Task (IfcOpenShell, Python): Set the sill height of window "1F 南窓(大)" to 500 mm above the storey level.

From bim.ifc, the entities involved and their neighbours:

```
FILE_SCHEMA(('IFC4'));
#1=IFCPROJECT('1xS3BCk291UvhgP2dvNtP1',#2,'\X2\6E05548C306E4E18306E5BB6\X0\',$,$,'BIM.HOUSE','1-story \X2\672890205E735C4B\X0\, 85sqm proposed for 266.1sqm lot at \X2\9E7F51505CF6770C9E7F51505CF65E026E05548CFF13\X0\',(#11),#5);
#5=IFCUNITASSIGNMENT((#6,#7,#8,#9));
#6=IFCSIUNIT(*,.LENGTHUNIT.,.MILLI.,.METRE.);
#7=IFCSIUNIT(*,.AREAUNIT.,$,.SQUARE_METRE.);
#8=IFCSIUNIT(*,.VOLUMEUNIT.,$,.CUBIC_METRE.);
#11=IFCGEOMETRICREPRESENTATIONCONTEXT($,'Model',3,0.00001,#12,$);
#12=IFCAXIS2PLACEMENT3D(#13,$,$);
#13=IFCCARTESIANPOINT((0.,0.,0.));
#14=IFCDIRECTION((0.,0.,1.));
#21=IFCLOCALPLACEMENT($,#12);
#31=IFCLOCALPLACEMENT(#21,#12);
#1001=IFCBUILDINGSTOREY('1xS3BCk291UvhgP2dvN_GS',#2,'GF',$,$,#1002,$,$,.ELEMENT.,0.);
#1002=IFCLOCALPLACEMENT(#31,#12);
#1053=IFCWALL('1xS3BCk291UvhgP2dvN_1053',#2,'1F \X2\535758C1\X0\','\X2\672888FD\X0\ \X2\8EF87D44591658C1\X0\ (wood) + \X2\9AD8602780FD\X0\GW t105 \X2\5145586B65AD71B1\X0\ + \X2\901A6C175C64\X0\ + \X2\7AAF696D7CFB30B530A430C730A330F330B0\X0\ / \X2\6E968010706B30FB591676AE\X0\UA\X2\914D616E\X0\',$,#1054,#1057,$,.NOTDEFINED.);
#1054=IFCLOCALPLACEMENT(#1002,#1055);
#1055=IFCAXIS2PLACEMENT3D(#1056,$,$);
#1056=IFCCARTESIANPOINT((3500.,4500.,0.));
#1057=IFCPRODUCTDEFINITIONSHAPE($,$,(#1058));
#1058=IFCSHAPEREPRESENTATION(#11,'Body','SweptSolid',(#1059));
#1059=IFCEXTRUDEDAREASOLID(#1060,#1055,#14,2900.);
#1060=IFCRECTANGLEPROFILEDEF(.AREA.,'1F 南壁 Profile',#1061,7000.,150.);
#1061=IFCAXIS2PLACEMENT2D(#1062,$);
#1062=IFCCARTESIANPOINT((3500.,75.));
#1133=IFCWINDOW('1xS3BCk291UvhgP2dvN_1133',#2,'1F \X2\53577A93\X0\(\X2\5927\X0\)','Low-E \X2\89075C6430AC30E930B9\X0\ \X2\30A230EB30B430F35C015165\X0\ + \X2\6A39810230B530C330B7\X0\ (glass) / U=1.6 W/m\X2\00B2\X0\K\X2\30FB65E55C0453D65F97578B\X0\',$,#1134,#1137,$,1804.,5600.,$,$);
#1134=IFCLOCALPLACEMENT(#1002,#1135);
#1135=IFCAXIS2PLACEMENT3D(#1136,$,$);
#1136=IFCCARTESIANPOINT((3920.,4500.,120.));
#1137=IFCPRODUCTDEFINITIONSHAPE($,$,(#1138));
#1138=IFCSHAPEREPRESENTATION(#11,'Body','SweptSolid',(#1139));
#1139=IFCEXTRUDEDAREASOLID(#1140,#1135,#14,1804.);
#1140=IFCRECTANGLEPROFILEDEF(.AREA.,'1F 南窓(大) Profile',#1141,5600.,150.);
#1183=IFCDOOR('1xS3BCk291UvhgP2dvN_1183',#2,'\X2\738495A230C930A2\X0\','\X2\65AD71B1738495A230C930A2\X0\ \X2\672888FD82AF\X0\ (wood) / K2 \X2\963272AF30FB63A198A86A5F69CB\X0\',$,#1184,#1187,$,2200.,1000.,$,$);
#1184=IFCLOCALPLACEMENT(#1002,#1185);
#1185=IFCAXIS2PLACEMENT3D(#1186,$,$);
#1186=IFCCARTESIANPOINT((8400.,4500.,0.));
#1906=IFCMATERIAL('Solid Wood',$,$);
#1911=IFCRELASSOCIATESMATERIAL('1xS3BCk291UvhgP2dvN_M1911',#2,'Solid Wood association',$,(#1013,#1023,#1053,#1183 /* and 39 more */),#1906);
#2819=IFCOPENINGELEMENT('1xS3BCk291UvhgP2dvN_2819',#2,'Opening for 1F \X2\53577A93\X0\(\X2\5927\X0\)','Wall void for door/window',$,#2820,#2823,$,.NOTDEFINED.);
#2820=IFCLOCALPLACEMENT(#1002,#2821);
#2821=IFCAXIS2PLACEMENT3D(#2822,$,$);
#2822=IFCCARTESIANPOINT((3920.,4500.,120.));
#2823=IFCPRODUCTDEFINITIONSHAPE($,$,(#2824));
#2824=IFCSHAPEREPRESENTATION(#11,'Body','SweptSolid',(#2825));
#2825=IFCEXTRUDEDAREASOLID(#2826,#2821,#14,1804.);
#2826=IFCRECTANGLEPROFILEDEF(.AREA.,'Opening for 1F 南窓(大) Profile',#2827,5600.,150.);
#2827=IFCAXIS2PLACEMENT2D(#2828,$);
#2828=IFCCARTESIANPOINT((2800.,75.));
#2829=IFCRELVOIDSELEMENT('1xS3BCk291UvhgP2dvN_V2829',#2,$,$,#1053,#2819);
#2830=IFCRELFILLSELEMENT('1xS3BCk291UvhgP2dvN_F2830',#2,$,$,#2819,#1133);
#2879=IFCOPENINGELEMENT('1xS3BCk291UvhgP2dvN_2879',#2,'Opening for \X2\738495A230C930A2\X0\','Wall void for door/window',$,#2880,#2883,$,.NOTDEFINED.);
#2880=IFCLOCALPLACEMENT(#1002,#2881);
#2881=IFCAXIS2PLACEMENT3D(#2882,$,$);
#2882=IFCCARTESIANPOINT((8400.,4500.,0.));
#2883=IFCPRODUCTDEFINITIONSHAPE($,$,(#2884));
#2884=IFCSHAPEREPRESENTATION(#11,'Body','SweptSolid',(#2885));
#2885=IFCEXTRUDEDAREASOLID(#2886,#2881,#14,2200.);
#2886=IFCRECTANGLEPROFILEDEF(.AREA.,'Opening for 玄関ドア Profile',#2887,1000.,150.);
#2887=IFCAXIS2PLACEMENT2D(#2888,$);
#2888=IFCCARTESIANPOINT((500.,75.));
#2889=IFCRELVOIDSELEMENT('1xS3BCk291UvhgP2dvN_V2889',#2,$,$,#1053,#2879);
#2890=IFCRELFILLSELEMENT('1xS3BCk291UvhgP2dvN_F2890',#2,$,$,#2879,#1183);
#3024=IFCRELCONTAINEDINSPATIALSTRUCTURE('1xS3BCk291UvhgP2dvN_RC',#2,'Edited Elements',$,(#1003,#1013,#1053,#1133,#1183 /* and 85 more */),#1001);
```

```python
import numpy as np
import ifcopenshell
import ifcopenshell.api.geometry
import ifcopenshell.geom
import ifcopenshell.util.element
import ifcopenshell.util.placement
import ifcopenshell.util.shape
import ifcopenshell.util.unit

model = ifcopenshell.open("bim.ifc")
unit_scale = ifcopenshell.util.unit.calculate_unit_scale(model)

window = model.by_id(1133)
opening = window.FillsVoids[0].RelatingOpeningElement
storey = ifcopenshell.util.element.get_container(window, ifc_class="IfcBuildingStorey")
level = ifcopenshell.util.placement.get_local_placement(storey.ObjectPlacement)[2, 3]

# The opening's origin need not be at the sill, so measure its lowest point.
shape = ifcopenshell.geom.create_shape(ifcopenshell.geom.settings(), opening)
bottom = ifcopenshell.util.shape.get_shape_bottom_elevation(shape, shape.geometry) / unit_scale
dz = level + 500.0 - bottom

shift = np.array([0.0, 0.0, dz])
# The window is not placed relative to its opening, so move both.
for product in (opening, window):
    matrix = ifcopenshell.util.placement.get_local_placement(product.ObjectPlacement)
    matrix[:3, 3] += shift
    ifcopenshell.api.geometry.edit_object_placement(model, product=product, matrix=matrix, is_si=False)

print(f"moved by {dz * unit_scale:+.3f} m")

model.write("bim_updated.ifc")
```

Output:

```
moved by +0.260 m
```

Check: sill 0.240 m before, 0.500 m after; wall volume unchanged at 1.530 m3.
